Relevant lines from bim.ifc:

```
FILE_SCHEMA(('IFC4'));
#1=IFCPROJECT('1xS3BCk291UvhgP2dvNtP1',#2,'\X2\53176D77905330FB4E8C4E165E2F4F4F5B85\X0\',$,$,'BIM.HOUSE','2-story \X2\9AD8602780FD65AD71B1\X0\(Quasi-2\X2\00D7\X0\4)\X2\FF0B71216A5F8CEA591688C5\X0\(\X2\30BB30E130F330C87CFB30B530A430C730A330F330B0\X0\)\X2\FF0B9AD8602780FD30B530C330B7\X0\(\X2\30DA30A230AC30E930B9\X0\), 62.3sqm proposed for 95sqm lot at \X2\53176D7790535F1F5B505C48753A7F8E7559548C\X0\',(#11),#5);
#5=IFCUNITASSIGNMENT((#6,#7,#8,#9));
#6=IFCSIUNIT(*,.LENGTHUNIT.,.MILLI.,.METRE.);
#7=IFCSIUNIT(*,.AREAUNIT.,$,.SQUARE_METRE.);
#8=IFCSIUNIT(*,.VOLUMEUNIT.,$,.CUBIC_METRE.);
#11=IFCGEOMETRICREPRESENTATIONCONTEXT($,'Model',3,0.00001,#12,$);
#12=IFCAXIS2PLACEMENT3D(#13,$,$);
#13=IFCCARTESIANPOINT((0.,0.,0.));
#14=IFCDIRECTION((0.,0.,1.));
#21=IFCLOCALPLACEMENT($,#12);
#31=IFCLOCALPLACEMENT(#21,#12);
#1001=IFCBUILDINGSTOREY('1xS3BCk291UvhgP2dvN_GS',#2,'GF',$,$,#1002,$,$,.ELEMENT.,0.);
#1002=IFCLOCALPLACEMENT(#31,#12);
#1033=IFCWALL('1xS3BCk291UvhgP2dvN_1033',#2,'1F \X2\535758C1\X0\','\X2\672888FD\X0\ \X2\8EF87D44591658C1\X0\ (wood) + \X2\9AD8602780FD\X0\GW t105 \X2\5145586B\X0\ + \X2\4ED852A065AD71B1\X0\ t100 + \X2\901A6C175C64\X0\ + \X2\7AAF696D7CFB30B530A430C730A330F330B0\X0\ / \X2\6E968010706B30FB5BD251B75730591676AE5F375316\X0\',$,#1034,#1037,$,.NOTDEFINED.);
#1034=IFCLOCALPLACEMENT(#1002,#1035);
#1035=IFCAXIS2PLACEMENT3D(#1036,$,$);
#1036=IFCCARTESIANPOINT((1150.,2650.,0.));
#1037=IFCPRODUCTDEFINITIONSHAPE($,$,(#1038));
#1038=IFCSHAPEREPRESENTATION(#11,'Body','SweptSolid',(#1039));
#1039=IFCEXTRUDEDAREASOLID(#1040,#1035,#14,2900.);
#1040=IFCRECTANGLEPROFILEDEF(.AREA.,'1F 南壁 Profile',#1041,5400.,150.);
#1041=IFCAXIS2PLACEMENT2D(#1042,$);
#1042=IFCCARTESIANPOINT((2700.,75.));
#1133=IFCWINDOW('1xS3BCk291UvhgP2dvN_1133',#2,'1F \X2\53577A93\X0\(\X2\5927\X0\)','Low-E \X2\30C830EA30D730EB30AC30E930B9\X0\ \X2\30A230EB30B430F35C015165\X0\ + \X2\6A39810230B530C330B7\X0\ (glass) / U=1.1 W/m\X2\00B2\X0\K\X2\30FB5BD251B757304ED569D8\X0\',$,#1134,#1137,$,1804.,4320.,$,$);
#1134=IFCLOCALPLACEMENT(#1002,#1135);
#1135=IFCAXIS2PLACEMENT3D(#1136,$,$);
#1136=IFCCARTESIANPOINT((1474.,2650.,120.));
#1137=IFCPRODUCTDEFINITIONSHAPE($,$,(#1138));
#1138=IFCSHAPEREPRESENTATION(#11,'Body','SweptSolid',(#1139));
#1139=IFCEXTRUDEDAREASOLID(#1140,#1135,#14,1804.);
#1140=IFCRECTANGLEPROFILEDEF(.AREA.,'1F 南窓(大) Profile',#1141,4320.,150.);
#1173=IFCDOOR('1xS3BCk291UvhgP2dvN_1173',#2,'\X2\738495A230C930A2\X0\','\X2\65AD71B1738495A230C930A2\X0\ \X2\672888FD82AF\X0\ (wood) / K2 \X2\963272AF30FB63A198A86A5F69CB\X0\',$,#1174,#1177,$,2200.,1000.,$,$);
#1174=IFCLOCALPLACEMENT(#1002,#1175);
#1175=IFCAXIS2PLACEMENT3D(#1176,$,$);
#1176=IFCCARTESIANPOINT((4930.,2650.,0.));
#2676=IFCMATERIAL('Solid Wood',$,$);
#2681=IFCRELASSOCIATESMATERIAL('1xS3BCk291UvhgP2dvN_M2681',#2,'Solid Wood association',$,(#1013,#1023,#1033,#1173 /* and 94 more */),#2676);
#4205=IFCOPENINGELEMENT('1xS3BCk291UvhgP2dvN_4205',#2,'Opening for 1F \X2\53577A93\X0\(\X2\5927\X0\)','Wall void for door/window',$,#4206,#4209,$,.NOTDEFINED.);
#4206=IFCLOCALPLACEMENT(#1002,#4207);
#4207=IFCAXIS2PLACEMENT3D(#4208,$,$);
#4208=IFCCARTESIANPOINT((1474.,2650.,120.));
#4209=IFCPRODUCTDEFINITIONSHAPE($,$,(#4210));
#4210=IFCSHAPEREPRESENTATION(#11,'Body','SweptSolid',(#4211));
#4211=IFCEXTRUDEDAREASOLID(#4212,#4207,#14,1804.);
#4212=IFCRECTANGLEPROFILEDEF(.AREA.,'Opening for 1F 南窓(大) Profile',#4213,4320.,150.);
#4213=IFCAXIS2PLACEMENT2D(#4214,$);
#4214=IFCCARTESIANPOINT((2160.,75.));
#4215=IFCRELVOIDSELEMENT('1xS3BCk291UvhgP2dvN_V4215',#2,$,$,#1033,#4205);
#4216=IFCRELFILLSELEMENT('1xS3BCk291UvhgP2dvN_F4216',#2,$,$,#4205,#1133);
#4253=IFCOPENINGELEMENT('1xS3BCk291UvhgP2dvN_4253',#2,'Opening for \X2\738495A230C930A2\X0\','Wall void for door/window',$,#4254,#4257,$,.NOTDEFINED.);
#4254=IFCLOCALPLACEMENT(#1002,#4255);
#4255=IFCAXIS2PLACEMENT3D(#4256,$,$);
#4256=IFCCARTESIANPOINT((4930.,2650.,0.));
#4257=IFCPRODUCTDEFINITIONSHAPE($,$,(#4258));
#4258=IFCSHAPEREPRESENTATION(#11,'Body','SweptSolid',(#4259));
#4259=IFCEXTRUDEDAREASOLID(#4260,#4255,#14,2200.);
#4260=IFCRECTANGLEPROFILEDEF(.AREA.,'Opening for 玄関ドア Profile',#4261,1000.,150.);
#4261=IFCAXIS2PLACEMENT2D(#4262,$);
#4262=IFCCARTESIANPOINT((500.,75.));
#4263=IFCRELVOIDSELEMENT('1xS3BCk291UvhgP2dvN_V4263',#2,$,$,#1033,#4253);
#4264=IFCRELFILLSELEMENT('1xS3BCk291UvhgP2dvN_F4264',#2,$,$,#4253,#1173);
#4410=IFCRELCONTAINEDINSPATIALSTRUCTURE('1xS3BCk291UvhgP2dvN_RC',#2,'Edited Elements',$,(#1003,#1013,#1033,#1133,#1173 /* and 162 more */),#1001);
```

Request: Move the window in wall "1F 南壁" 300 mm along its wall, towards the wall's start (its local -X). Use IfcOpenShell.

```python
import ifcopenshell
import ifcopenshell.api.geometry
import ifcopenshell.util.placement

model = ifcopenshell.open("bim.ifc")

window = model.by_id(1133)
opening = window.FillsVoids[0].RelatingOpeningElement
wall = opening.VoidsElements[0].RelatingBuildingElement

wall_matrix = ifcopenshell.util.placement.get_local_placement(wall.ObjectPlacement)
shift = wall_matrix[:3, 0] * -300.0
before = ifcopenshell.util.placement.get_local_placement(window.ObjectPlacement)[:3, 3].copy()

# The window is not placed relative to its opening, so move both.
for product in (opening, window):
    matrix = ifcopenshell.util.placement.get_local_placement(product.ObjectPlacement)
    matrix[:3, 3] += shift
    ifcopenshell.api.geometry.edit_object_placement(model, product=product, matrix=matrix, is_si=False)

after = ifcopenshell.util.placement.get_local_placement(window.ObjectPlacement)[:3, 3]
print("window moved by", (after - before).round(3) + 0.0)

model.write("bim_v2.ifc")
```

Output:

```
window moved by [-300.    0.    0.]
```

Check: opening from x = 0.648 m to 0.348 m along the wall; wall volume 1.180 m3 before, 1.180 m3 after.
